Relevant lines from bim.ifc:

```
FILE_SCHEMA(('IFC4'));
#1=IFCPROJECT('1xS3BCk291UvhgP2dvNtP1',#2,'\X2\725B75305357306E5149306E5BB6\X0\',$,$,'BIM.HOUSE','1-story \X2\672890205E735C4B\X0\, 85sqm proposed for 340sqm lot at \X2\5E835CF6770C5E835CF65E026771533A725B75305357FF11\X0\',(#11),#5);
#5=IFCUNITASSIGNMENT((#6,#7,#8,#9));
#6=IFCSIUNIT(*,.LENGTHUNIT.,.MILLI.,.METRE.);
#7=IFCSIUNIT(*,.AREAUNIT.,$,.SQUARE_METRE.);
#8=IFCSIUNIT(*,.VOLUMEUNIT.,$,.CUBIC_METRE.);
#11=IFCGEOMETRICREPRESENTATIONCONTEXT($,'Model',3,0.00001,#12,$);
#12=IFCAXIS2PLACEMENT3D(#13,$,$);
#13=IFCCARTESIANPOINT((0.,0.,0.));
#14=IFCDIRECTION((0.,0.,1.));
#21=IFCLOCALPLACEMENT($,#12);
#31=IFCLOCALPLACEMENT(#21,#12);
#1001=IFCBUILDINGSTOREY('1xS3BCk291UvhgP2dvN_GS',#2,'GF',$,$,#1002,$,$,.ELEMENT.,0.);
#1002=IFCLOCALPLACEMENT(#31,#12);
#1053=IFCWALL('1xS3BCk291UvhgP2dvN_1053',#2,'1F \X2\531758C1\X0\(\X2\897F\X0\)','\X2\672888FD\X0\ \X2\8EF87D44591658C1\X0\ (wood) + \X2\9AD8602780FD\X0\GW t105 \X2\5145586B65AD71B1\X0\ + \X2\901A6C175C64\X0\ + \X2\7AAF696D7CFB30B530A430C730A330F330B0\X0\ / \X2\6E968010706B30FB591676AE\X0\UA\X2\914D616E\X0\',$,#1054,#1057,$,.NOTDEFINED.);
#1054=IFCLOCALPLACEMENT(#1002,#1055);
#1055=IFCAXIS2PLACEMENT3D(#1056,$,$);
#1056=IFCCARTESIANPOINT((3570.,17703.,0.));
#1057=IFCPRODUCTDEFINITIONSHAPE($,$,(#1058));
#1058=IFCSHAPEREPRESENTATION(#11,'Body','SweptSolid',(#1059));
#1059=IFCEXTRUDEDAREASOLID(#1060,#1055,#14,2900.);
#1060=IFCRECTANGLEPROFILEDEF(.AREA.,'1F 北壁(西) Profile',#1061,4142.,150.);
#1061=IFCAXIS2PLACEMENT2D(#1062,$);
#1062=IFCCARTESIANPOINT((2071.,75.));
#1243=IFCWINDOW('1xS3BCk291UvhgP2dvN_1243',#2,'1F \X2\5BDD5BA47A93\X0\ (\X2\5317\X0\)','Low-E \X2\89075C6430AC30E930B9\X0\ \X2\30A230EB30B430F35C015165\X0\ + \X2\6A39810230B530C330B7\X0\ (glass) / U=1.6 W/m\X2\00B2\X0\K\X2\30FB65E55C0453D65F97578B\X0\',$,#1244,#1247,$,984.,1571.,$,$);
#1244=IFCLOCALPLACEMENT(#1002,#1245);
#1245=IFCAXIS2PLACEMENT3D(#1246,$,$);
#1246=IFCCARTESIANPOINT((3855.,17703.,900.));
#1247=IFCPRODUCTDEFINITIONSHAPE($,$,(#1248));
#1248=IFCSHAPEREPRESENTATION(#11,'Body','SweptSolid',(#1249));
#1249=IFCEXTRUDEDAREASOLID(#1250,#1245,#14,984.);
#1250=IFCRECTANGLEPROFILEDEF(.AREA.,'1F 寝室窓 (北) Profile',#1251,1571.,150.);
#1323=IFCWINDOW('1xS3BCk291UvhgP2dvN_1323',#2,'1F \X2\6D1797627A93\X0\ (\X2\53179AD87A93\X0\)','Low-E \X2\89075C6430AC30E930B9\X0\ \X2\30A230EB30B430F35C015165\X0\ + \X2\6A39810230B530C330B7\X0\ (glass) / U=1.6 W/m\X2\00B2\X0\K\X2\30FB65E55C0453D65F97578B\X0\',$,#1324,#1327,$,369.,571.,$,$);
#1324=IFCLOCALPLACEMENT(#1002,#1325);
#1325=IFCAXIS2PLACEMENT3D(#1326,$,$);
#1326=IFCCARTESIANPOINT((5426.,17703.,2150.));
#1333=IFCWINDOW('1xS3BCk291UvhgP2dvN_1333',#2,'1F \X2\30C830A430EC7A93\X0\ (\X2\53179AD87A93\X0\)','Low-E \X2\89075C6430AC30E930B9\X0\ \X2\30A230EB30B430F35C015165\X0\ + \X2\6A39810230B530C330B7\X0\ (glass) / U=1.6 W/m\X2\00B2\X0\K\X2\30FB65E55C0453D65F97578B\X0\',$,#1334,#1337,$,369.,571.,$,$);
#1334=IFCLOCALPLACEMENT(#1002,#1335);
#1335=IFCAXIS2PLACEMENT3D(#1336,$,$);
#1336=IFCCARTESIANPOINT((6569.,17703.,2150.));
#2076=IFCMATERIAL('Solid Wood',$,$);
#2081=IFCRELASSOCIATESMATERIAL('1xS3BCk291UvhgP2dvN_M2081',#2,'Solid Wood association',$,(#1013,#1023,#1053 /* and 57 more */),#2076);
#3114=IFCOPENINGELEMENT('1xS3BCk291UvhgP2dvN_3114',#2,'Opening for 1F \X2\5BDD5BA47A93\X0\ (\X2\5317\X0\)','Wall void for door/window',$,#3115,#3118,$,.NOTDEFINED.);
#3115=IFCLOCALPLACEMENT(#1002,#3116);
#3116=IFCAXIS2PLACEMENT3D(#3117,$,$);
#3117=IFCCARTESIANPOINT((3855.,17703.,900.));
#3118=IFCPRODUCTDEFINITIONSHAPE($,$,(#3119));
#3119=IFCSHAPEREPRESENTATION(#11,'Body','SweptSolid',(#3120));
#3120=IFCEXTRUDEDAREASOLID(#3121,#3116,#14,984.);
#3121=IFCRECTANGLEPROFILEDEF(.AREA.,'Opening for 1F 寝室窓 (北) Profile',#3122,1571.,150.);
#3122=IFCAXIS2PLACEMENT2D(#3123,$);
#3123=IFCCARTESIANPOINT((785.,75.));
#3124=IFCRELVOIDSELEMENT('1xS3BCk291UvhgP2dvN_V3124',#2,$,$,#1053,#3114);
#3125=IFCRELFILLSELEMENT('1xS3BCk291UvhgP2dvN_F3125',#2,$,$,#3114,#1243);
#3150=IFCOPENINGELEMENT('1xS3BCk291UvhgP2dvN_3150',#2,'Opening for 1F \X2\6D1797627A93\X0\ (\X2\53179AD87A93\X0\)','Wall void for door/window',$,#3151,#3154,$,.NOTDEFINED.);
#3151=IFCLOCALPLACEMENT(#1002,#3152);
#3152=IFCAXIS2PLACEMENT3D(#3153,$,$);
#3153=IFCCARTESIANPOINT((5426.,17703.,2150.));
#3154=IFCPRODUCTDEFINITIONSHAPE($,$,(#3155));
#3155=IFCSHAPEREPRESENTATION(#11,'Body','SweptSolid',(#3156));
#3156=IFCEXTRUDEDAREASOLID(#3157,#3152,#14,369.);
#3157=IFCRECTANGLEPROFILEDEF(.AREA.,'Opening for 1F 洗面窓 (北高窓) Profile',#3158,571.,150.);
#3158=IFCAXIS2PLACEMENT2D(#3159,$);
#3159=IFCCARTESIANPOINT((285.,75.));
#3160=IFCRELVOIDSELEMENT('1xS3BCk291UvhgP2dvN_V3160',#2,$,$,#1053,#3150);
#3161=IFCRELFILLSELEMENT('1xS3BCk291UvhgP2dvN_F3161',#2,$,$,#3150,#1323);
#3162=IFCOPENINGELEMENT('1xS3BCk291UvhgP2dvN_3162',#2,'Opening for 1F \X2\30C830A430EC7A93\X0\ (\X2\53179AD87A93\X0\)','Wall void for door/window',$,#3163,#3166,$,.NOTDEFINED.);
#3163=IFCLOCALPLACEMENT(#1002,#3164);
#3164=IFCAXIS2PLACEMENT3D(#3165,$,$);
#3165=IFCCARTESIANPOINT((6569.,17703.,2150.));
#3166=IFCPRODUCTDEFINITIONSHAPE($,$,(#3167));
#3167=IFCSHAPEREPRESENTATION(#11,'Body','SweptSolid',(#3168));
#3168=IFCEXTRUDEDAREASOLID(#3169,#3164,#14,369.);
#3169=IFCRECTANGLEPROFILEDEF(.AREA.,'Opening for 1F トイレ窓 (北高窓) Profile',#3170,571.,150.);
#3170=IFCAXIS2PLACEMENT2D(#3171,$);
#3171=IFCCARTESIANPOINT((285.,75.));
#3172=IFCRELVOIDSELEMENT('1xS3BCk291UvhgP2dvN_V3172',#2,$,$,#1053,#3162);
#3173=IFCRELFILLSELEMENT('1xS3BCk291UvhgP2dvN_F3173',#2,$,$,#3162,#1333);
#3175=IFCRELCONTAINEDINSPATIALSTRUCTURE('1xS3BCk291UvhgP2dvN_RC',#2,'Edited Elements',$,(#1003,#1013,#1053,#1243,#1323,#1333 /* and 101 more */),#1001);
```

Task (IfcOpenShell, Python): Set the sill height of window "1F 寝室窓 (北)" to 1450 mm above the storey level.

```python
import numpy as np
import ifcopenshell
import ifcopenshell.api.geometry
import ifcopenshell.geom
import ifcopenshell.util.element
import ifcopenshell.util.placement
import ifcopenshell.util.shape
import ifcopenshell.util.unit

model = ifcopenshell.open("bim.ifc")
unit_scale = ifcopenshell.util.unit.calculate_unit_scale(model)

window = model.by_guid("1xS3BCk291UvhgP2dvN_1243")
opening = window.FillsVoids[0].RelatingOpeningElement
storey = ifcopenshell.util.element.get_container(window, ifc_class="IfcBuildingStorey")
level = ifcopenshell.util.placement.get_local_placement(storey.ObjectPlacement)[2, 3]

# The opening's origin need not be at the sill, so measure its lowest point.
shape = ifcopenshell.geom.create_shape(ifcopenshell.geom.settings(), opening)
bottom = ifcopenshell.util.shape.get_shape_bottom_elevation(shape, shape.geometry) / unit_scale
dz = level + 1.45 / unit_scale - bottom

shift = np.array([0.0, 0.0, dz])
# The window is not placed relative to its opening, so move both.
for product in (opening, window):
    matrix = ifcopenshell.util.placement.get_local_placement(product.ObjectPlacement)
    matrix[:3, 3] += shift
    ifcopenshell.api.geometry.edit_object_placement(model, product=product, matrix=matrix, is_si=False)

print(f"moved by {dz * unit_scale:+.3f} m")

model.write("bim_edited.ifc")
```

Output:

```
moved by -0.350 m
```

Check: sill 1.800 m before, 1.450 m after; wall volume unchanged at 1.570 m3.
